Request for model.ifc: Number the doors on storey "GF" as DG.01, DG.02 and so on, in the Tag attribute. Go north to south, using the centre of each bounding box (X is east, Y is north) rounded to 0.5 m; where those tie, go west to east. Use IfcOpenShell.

First a look at what the model holds.

```python
import ifcopenshell
import ifcopenshell.util.element
import ifcopenshell.util.placement

model = ifcopenshell.open("model.ifc")
print(model.schema)
storey = next(s for s in model.by_type("IfcBuildingStorey") if s.Name == "GF")
doors = [e for e in ifcopenshell.util.element.get_decomposition(storey) if e.is_a("IfcDoor")]
for e in sorted(doors, key=lambda e: e.id()):
    origin = ifcopenshell.util.placement.get_local_placement(e.ObjectPlacement)[:3, 3]
    print(e.id(), e.Tag, e.Name, origin.round(2) + 0.0, sep=" | ")
```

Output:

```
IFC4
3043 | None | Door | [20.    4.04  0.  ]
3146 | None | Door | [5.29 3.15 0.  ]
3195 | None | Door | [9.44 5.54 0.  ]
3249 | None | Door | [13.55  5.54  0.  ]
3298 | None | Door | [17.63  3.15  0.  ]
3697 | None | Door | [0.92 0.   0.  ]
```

```python
import ifcopenshell
import ifcopenshell.geom
import ifcopenshell.util.element
import ifcopenshell.util.shape

model = ifcopenshell.open("model.ifc")
settings = ifcopenshell.geom.settings()
settings.set("use-world-coords", True)


def centre(element):
    shape = ifcopenshell.geom.create_shape(settings, element)
    return ifcopenshell.util.shape.get_bbox_centroid(shape.geometry)


storey = next(s for s in model.by_type("IfcBuildingStorey") if s.Name == "GF")
doors = [e for e in ifcopenshell.util.element.get_decomposition(storey) if e.is_a("IfcDoor")]

# Insertion points can sit at a corner or the storey origin, so sort by the geometry (in metres).
centres = {e: centre(e) for e in doors}
doors.sort(key=lambda e: (-round(centres[e][1] / 0.5), centres[e][0]))

for i, e in enumerate(doors, start=1):
    number = f"DG.{i:02d}"
    e.Tag = number
    print(e.id(), number)

model.write("model_edited.ifc")
```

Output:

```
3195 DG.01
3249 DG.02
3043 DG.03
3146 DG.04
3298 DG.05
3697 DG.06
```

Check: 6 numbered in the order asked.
